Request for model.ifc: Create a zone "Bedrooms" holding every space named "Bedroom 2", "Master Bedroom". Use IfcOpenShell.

First a look at what the model holds.

```python
import ifcopenshell

model = ifcopenshell.open("model.ifc")
print(model.schema)
seen = {}
for space in model.by_type("IfcSpace"):
    seen[space.LongName] = seen.get(space.LongName, 0) + 1
for name, count in sorted(seen.items(), key=str):
    print(count, "x", name)
print("zones:", [z.Name for z in model.by_type("IfcZone")][:20])
```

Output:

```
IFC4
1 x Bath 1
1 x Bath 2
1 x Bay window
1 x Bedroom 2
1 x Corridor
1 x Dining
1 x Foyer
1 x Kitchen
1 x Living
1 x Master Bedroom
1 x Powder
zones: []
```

```python
import ifcopenshell
import ifcopenshell.api.group
import ifcopenshell.api.root

model = ifcopenshell.open("model.ifc")

names = {"Bedroom 2", "Master Bedroom"}
spaces = [s for s in model.by_type("IfcSpace") if s.LongName in names]

zone = ifcopenshell.api.root.create_entity(model, ifc_class="IfcZone", name="Bedrooms")
ifcopenshell.api.group.assign_group(model, products=spaces, group=zone)
print(len(spaces), "spaces in", zone.Name)

model.write("model_edited.ifc")
```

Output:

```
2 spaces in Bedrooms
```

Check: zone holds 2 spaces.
